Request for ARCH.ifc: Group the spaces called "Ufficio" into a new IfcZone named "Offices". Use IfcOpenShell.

First a look at what the model holds.

```python
import ifcopenshell

model = ifcopenshell.open("ARCH.ifc")
print(model.schema)
seen = {}
for space in model.by_type("IfcSpace"):
    seen[space.LongName] = seen.get(space.LongName, 0) + 1
for name, count in sorted(seen.items(), key=str):
    print(count, "x", name)
print("zones:", [z.Name for z in model.by_type("IfcZone")][:20])
```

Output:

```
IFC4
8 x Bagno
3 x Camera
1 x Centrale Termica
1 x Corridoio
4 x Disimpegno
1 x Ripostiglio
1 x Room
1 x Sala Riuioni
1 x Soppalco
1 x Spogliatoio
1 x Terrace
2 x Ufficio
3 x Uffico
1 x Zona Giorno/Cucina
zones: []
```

```python
import ifcopenshell
import ifcopenshell.api.group
import ifcopenshell.api.root

model = ifcopenshell.open("ARCH.ifc")

names = {"Ufficio"}
spaces = [s for s in model.by_type("IfcSpace") if s.LongName in names]

zone = ifcopenshell.api.root.create_entity(model, ifc_class="IfcZone", name="Offices")
ifcopenshell.api.group.assign_group(model, products=spaces, group=zone)
print(len(spaces), "spaces in", zone.Name)

model.write("ARCH_rev.ifc")
```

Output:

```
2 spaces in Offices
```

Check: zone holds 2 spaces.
